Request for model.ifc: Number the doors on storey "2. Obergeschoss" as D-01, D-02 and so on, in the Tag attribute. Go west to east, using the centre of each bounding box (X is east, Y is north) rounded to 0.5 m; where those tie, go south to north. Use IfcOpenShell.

First a look at what the model holds.

```python
import ifcopenshell
import ifcopenshell.util.element
import ifcopenshell.util.placement

model = ifcopenshell.open("model.ifc")
print(model.schema)
storey = next(s for s in model.by_type("IfcBuildingStorey") if s.Name == "2. Obergeschoss")
doors = [e for e in ifcopenshell.util.element.get_decomposition(storey) if e.is_a("IfcDoor")]
for e in sorted(doors, key=lambda e: e.id()):
    origin = ifcopenshell.util.placement.get_local_placement(e.ObjectPlacement)[:3, 3]
    print(e.id(), e.Tag, e.Name, origin.round(2) + 0.0, sep=" | ")
```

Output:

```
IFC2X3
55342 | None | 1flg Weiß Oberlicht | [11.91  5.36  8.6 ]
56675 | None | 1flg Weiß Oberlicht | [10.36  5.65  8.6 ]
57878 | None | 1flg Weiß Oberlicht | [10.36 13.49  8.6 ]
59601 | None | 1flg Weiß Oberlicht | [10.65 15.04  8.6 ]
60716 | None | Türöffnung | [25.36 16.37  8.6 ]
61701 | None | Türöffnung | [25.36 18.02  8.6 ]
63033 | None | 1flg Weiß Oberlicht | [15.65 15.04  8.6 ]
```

```python
import ifcopenshell
import ifcopenshell.geom
import ifcopenshell.util.element
import ifcopenshell.util.shape

model = ifcopenshell.open("model.ifc")
settings = ifcopenshell.geom.settings()
settings.set("use-world-coords", True)


def centre(element):
    shape = ifcopenshell.geom.create_shape(settings, element)
    return ifcopenshell.util.shape.get_bbox_centroid(shape.geometry)


storey = next(s for s in model.by_type("IfcBuildingStorey") if s.Name == "2. Obergeschoss")
doors = [e for e in ifcopenshell.util.element.get_decomposition(storey) if e.is_a("IfcDoor")]

# Insertion points can sit at a corner or the storey origin, so sort by the geometry (in metres).
centres = {e: centre(e) for e in doors}
doors.sort(key=lambda e: (round(centres[e][0] / 0.5), centres[e][1]))

for i, e in enumerate(doors, start=1):
    number = f"D-{i:02d}"
    e.Tag = number
    print(e.id(), number)

model.write("model_v2.ifc")
```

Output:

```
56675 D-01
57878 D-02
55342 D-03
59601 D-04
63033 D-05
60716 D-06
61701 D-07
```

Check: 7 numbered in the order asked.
